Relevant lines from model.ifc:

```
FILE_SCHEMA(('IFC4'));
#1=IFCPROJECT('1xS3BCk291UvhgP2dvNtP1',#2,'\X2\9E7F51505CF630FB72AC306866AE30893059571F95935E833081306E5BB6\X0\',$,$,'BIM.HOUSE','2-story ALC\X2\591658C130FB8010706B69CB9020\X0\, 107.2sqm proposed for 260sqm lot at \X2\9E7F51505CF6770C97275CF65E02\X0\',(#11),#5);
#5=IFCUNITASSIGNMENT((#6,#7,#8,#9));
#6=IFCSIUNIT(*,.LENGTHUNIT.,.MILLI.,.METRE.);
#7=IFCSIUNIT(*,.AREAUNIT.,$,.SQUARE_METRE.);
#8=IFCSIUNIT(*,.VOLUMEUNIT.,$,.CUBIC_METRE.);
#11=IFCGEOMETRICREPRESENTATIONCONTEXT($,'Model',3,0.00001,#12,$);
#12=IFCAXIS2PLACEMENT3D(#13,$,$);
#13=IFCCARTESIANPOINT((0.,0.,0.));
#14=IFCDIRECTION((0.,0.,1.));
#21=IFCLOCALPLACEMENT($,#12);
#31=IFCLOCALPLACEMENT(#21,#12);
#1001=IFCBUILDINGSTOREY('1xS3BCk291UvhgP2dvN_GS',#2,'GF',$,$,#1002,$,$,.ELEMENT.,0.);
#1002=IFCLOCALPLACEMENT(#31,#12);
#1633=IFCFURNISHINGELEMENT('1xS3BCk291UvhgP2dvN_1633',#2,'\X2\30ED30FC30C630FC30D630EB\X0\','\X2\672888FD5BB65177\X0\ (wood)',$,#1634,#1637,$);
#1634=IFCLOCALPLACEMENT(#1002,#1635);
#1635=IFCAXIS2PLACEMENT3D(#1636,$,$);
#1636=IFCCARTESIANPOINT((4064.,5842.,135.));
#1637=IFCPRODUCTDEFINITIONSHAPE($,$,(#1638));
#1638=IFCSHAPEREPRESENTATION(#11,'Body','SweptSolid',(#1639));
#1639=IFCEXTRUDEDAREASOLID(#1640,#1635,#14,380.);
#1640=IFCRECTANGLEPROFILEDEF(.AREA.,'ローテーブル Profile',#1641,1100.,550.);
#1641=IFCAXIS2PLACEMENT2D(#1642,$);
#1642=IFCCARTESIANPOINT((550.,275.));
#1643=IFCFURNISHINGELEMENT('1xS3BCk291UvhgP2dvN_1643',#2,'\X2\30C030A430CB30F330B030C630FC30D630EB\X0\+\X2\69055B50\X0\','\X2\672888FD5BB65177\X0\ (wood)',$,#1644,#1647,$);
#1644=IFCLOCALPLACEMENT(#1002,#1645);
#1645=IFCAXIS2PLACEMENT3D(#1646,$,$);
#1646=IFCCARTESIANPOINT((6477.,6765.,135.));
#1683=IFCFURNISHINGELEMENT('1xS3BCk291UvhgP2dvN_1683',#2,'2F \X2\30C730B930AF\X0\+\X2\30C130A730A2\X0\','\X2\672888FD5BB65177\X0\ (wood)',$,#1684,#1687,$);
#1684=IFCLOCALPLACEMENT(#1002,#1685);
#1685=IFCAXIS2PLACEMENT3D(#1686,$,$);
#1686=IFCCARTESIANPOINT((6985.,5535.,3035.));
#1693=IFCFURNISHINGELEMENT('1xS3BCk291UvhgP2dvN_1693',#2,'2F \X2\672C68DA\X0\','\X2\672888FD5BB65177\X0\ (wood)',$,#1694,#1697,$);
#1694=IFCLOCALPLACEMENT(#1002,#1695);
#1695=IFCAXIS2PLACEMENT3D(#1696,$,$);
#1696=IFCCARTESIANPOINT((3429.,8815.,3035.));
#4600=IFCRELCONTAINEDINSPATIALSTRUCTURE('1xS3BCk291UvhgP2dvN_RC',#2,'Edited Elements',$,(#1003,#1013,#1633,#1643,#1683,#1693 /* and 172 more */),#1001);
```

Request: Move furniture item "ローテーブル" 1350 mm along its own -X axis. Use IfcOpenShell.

```python
import ifcopenshell
import ifcopenshell.api.geometry
import ifcopenshell.util.placement
import ifcopenshell.util.unit

model = ifcopenshell.open("model.ifc")
unit_scale = ifcopenshell.util.unit.calculate_unit_scale(model)

item = model.by_guid("1xS3BCk291UvhgP2dvN_1633")
matrix = ifcopenshell.util.placement.get_local_placement(item.ObjectPlacement)
matrix[:3, 3] -= matrix[:3, 0] * 1.35 / unit_scale
ifcopenshell.api.geometry.edit_object_placement(model, product=item, matrix=matrix, is_si=False)

print(ifcopenshell.util.placement.get_local_placement(item.ObjectPlacement).round(3) + 0.0)

model.write("model_v2.ifc")
```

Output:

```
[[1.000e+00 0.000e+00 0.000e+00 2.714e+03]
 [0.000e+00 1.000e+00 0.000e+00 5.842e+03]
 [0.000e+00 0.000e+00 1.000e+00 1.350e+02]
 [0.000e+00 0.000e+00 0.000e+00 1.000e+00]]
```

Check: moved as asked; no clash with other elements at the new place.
